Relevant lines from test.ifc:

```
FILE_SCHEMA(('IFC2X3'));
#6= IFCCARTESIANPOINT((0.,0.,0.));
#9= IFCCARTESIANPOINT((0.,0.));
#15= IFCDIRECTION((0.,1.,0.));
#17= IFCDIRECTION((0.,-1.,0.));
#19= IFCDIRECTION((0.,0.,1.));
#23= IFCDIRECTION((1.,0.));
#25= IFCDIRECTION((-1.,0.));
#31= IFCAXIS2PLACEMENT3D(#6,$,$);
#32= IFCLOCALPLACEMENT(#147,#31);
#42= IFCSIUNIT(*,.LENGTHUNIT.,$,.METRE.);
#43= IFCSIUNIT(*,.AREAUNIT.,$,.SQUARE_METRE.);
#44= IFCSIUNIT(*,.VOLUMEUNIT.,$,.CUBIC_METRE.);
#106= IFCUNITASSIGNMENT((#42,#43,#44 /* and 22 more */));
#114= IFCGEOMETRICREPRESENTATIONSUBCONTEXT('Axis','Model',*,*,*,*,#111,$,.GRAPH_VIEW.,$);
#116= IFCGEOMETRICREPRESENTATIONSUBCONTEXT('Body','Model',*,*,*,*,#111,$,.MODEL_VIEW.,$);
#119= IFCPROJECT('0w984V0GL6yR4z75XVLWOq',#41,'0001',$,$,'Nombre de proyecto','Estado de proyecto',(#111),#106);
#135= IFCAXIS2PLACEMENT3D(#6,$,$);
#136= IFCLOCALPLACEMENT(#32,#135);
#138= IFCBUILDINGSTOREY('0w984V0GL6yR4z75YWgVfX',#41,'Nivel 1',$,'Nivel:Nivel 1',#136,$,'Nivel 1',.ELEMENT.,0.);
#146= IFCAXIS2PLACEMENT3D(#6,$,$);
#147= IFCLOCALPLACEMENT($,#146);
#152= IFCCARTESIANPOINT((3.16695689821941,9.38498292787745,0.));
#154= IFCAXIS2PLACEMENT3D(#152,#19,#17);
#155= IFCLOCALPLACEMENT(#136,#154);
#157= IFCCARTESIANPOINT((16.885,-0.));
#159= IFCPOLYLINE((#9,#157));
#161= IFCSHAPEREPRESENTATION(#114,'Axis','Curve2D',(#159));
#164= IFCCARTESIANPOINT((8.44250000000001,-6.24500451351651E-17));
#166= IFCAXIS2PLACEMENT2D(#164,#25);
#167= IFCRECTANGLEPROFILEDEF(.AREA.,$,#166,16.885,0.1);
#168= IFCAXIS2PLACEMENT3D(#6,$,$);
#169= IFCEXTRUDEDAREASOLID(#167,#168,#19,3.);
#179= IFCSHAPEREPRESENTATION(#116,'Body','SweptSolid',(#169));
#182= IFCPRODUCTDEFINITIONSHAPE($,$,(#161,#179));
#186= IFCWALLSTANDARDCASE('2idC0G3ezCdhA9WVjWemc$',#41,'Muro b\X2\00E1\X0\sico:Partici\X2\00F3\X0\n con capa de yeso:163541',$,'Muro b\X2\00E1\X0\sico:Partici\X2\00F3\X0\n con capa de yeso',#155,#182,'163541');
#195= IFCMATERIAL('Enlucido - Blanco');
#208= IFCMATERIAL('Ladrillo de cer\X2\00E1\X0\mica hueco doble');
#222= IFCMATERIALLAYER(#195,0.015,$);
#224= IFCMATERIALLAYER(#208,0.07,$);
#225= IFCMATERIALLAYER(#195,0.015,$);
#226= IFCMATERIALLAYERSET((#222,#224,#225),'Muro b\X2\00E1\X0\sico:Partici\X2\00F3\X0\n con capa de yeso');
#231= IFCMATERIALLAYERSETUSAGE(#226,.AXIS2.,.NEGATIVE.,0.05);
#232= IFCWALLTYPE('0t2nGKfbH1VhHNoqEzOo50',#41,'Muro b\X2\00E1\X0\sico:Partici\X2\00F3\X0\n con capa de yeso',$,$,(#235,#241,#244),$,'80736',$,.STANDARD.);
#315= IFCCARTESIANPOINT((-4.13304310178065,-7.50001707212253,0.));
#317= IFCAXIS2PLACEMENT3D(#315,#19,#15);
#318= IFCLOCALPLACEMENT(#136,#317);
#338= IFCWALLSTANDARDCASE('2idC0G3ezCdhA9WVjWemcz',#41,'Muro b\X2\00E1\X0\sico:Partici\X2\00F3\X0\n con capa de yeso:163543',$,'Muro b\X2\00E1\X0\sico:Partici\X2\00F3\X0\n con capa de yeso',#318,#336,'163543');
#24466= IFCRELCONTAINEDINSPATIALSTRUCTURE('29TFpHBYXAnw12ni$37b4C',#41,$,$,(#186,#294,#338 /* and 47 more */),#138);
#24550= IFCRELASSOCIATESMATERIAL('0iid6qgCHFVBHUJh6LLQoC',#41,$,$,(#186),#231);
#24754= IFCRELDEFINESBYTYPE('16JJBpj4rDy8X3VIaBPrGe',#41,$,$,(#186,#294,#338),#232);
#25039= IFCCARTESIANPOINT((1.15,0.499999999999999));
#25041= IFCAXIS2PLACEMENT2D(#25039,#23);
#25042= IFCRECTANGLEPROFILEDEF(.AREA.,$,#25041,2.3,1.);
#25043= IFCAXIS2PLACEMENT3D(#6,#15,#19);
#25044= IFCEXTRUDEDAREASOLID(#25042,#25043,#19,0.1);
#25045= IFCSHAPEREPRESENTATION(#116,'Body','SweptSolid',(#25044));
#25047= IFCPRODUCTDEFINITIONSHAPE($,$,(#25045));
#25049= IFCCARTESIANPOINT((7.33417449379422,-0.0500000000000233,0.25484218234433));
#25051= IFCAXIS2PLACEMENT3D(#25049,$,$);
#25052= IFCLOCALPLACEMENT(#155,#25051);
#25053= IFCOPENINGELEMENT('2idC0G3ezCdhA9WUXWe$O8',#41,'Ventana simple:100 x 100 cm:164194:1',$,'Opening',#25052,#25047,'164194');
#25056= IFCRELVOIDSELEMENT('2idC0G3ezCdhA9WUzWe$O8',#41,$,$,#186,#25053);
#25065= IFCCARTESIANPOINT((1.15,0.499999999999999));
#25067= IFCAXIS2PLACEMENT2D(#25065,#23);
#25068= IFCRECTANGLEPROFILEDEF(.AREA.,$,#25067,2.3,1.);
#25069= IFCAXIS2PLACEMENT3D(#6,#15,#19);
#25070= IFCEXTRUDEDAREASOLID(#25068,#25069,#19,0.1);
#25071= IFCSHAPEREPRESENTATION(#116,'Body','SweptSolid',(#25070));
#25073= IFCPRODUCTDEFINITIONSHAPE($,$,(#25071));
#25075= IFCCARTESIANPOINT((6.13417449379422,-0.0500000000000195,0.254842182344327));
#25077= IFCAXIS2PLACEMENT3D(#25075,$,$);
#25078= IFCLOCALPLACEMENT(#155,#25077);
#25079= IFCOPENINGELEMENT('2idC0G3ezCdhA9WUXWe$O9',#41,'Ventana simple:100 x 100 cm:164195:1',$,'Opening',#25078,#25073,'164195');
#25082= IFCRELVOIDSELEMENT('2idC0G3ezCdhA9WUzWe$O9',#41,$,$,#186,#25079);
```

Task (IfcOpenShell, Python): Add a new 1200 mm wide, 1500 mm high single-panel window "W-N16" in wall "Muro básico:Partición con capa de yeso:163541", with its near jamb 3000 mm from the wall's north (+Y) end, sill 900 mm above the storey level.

```python
import numpy as np
import ifcopenshell
import ifcopenshell.api.feature
import ifcopenshell.api.geometry
import ifcopenshell.api.root
import ifcopenshell.api.spatial
import ifcopenshell.api.type
import ifcopenshell.geom
import ifcopenshell.util.element
import ifcopenshell.util.placement
import ifcopenshell.util.representation
import ifcopenshell.util.shape
import ifcopenshell.util.unit

model = ifcopenshell.open("test.ifc")
unit_scale = ifcopenshell.util.unit.calculate_unit_scale(model)
settings = ifcopenshell.geom.settings()


def volume(element):
    """Net volume in cubic metres, openings subtracted."""
    shape = ifcopenshell.geom.create_shape(settings, element)
    return ifcopenshell.util.shape.get_volume(shape.geometry)


wall = model.by_guid("2idC0G3ezCdhA9WVjWemc$")
storey = ifcopenshell.util.element.get_container(wall, ifc_class="IfcBuildingStorey")
context = ifcopenshell.util.representation.get_context(model, "Model", "Body", "MODEL_VIEW")
before = volume(wall)

width, height, from_end, sill = 1.2, 1.5, 3, 0.9  # metres

# The wall runs along its own X axis, and the end named is its -X end.
wall_shape = ifcopenshell.geom.create_shape(settings, wall)
x, y, z = ifcopenshell.util.shape.get_vertices(wall_shape.geometry).T
start = x.min() + from_end
face, thickness = float(y.min()), float(y.max() - y.min())
wall_matrix = ifcopenshell.util.placement.get_local_placement(wall.ObjectPlacement)
level = ifcopenshell.util.placement.get_local_placement(storey.ObjectPlacement)[2, 3]


def in_wall(x, y):
    """Placement at x, y metres in the wall's axes, at sill height."""
    matrix = wall_matrix.copy()
    matrix[:, 3] = wall_matrix @ np.array([x / unit_scale, y / unit_scale, 0.0, 1.0])
    matrix[2, 3] = level + sill / unit_scale
    return matrix


# Opening: a box that overshoots both wall faces by 50 mm.
opening = ifcopenshell.api.root.create_entity(model, ifc_class="IfcOpeningElement")
box = ifcopenshell.api.geometry.add_wall_representation(
    model, context=context, length=width, height=height, thickness=thickness + 0.1
)
ifcopenshell.api.geometry.assign_representation(model, product=opening, representation=box)
ifcopenshell.api.geometry.edit_object_placement(model, product=opening, matrix=in_wall(start, face - 0.05), is_si=False)
ifcopenshell.api.feature.add_feature(model, feature=opening, element=wall)

window = ifcopenshell.api.root.create_entity(model, ifc_class="IfcWindow", name="W-N16")
window.OverallWidth, window.OverallHeight = width / unit_scale, height / unit_scale
body = ifcopenshell.api.geometry.add_window_representation(
    model,
    context=context,
    overall_width=window.OverallWidth,
    overall_height=window.OverallHeight,
    partition_type="SINGLE_PANEL",
)
ifcopenshell.api.geometry.assign_representation(model, product=window, representation=body)
ifcopenshell.api.spatial.assign_container(model, products=[window], relating_structure=storey)
fills = ifcopenshell.api.feature.add_filling(model, opening=opening, element=window)
fills.OwnerHistory = window.OwnerHistory  # required in IFC2X3

# IFC2X3 keeps the operation on the window style.
style = ifcopenshell.api.root.create_entity(model, ifc_class="IfcWindowStyle", name="W-N16")
style.OperationType, style.ConstructionType = "SINGLE_PANEL", "NOTDEFINED"
style.ParameterTakesPrecedence = style.Sizeable = False
ifcopenshell.api.type.assign_type(model, related_objects=[window], relating_type=style)

# Centre the window in the wall's thickness.
ifcopenshell.api.geometry.edit_object_placement(model, product=window, matrix=in_wall(start, face), is_si=False)
window_shape = ifcopenshell.geom.create_shape(settings, window)
depth = ifcopenshell.util.shape.get_vertices(window_shape.geometry)[:, 1]
offset = face + thickness / 2 - (depth.min() + depth.max()) / 2
ifcopenshell.api.geometry.edit_object_placement(model, product=window, matrix=in_wall(start, offset), is_si=False)

after = volume(wall)

print(f"wall volume {before:.3f} -> {after:.3f} m3")

model.write("test_rev.ifc")
```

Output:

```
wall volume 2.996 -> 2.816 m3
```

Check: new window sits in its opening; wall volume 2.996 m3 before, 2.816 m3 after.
